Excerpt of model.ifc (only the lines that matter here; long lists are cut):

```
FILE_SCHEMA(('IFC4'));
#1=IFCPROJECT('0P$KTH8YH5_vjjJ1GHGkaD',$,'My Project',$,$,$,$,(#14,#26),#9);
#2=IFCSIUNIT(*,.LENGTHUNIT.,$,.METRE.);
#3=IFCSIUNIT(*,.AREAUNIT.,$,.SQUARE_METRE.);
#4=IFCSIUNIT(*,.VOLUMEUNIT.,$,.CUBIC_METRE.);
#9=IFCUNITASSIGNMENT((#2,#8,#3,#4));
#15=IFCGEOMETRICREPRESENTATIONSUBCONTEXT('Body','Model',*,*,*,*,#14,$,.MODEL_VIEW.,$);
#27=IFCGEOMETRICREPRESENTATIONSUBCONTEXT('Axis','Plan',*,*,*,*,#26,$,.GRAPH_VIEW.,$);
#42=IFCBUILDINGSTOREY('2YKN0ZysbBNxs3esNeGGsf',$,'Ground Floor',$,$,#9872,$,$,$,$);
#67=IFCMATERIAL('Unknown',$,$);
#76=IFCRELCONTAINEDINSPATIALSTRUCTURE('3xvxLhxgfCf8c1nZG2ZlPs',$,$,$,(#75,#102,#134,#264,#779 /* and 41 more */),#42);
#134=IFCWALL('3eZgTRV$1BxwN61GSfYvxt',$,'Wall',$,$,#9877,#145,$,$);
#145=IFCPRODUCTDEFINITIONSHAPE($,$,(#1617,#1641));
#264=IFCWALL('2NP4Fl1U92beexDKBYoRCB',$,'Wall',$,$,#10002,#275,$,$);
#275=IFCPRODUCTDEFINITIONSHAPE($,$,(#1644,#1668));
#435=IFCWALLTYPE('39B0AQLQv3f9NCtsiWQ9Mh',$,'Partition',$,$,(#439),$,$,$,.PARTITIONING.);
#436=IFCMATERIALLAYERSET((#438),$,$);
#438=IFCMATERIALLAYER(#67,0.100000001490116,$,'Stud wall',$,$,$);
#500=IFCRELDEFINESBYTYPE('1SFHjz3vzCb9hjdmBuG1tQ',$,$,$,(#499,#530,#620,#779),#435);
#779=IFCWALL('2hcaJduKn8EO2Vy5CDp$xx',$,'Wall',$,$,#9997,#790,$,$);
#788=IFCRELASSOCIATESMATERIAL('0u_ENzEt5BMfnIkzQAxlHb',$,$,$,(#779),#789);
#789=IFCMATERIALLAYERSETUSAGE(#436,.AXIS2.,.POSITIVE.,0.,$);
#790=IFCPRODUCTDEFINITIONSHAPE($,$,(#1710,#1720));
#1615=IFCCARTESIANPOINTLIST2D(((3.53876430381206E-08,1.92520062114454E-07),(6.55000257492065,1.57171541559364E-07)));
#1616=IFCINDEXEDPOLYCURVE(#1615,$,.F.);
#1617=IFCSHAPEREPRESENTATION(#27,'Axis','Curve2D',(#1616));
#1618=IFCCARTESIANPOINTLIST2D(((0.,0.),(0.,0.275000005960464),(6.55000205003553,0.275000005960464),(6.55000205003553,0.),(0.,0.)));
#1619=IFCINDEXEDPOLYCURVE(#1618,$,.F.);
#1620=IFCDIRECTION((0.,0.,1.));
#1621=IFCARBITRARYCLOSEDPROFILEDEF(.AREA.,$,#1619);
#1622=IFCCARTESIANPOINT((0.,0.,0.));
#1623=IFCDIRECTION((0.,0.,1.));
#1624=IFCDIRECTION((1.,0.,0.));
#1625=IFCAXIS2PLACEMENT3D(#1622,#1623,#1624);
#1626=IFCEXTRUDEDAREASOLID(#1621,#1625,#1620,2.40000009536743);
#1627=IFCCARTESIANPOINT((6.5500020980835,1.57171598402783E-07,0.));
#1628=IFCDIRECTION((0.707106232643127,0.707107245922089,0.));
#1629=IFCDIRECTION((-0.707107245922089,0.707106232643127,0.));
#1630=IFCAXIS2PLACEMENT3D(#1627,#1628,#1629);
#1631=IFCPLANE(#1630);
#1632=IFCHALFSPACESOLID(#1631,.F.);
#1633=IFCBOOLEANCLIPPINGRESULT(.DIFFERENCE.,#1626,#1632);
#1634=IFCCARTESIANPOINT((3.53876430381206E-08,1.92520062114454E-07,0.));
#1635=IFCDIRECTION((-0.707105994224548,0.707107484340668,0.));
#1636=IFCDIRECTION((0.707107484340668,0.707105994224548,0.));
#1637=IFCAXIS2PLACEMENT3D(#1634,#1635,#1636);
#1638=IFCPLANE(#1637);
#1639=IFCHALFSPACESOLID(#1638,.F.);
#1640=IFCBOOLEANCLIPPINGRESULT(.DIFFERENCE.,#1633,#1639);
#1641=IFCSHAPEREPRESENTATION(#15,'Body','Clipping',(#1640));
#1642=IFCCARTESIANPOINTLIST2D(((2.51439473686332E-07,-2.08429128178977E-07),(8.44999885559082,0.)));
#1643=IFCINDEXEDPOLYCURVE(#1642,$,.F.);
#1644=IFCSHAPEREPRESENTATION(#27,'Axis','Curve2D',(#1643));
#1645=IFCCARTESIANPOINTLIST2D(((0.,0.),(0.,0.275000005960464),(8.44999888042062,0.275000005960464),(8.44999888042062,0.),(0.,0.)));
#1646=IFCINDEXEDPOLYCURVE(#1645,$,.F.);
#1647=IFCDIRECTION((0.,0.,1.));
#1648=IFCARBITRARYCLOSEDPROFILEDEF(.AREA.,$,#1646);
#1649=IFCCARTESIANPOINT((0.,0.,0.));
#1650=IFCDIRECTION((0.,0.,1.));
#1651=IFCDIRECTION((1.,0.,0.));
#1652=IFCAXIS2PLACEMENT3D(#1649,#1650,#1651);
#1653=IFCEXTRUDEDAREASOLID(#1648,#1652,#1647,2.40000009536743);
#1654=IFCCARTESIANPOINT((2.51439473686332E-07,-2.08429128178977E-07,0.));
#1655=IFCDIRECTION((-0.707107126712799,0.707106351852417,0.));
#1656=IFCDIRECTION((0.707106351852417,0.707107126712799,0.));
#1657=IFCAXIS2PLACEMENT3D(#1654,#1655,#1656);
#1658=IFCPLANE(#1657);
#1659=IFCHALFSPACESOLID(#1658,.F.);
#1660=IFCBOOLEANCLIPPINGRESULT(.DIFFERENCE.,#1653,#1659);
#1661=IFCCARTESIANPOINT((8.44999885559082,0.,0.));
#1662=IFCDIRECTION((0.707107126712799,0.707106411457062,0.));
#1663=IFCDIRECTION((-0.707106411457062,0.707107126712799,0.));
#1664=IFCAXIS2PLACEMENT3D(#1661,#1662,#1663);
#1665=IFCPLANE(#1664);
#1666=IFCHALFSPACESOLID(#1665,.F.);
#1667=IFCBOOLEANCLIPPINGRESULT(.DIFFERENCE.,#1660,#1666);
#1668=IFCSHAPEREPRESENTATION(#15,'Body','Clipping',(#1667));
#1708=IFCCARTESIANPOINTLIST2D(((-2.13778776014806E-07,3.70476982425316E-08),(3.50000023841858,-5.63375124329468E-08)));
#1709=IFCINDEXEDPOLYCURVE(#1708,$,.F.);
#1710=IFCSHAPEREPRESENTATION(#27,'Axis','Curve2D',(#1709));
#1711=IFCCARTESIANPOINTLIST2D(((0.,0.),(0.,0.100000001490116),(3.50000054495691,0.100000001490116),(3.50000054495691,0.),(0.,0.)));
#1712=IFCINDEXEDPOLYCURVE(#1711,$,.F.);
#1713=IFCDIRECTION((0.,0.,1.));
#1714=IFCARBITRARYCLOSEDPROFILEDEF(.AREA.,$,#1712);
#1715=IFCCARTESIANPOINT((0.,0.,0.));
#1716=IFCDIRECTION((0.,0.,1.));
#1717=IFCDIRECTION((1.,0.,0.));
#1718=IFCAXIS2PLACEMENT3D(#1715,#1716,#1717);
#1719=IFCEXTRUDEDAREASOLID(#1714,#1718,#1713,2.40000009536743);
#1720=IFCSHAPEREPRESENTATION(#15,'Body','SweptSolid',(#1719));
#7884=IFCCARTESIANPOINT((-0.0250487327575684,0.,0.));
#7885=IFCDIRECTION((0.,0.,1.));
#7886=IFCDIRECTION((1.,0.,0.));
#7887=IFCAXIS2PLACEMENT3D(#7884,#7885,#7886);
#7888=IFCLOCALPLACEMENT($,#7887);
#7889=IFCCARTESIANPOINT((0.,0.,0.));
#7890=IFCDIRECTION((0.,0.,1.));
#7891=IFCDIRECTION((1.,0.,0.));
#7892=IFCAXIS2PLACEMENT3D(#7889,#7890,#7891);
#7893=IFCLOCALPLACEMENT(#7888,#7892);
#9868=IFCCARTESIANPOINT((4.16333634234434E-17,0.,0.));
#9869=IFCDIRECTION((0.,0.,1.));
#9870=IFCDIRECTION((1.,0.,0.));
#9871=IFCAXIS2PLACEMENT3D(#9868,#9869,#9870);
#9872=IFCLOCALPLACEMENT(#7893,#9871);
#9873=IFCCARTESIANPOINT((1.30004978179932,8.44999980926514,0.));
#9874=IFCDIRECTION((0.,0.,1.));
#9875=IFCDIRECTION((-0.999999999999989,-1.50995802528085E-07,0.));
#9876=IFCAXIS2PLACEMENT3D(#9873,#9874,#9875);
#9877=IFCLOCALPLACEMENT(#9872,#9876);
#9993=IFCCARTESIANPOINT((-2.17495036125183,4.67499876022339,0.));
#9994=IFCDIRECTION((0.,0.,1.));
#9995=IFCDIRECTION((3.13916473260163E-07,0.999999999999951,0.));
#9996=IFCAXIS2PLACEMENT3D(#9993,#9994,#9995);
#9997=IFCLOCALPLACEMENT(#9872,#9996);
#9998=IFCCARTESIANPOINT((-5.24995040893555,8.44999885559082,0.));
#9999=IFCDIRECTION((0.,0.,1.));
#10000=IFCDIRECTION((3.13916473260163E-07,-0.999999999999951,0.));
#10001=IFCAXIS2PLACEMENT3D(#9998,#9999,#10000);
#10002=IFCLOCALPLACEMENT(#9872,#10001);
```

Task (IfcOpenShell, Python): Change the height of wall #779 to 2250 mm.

```python
import ifcopenshell
import ifcopenshell.geom
import ifcopenshell.util.representation
import ifcopenshell.util.shape

model = ifcopenshell.open("model.ifc")
settings = ifcopenshell.geom.settings()


def volume(element):
    """Net volume in cubic metres, openings subtracted."""
    shape = ifcopenshell.geom.create_shape(settings, element)
    return ifcopenshell.util.shape.get_volume(shape.geometry)


wall = model.by_guid("2hcaJduKn8EO2Vy5CDp$xx")
before = volume(wall)

body = ifcopenshell.util.representation.get_representation(wall, "Model", "Body")
solid = body.Items[0]
old_height = solid.Depth
solid.Depth = 2.25
after = volume(wall)

print(f"height {old_height:g} -> {solid.Depth:g}, volume {before:.3f} -> {after:.3f} m3")

model.write("model_v2.ifc")
```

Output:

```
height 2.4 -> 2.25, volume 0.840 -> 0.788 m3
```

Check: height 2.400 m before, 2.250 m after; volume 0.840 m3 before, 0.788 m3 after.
